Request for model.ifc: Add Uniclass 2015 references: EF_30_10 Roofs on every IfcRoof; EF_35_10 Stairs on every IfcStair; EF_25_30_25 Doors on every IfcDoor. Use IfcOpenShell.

First a look at what the model holds.

```python
import ifcopenshell

model = ifcopenshell.open("model.ifc")
print(model.schema)
print("classifications:", [c.Name for c in model.by_type("IfcClassification")])
for ifc_class in ("IfcDoor", "IfcRoof", "IfcStair", "IfcWall", "IfcWindow"):
    print(ifc_class, len(model.by_type(ifc_class)))
```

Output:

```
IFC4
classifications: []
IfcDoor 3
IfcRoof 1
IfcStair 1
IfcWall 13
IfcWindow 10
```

```python
import ifcopenshell
import ifcopenshell.api.classification

model = ifcopenshell.open("model.ifc")

system = ifcopenshell.api.classification.add_classification(model, classification="Uniclass 2015")

codes = {
    "IfcRoof": ("EF_30_10", "Roofs"),
    "IfcStair": ("EF_35_10", "Stairs"),
    "IfcDoor": ("EF_25_30_25", "Doors"),
}
for ifc_class, (code, name) in codes.items():
    products = model.by_type(ifc_class)
    ifcopenshell.api.classification.add_reference(
        model, products=products, classification=system, identification=code, name=name
    )
    print(code, len(products))

model.write("model_updated.ifc")
```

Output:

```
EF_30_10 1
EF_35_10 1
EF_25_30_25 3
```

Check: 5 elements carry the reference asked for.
